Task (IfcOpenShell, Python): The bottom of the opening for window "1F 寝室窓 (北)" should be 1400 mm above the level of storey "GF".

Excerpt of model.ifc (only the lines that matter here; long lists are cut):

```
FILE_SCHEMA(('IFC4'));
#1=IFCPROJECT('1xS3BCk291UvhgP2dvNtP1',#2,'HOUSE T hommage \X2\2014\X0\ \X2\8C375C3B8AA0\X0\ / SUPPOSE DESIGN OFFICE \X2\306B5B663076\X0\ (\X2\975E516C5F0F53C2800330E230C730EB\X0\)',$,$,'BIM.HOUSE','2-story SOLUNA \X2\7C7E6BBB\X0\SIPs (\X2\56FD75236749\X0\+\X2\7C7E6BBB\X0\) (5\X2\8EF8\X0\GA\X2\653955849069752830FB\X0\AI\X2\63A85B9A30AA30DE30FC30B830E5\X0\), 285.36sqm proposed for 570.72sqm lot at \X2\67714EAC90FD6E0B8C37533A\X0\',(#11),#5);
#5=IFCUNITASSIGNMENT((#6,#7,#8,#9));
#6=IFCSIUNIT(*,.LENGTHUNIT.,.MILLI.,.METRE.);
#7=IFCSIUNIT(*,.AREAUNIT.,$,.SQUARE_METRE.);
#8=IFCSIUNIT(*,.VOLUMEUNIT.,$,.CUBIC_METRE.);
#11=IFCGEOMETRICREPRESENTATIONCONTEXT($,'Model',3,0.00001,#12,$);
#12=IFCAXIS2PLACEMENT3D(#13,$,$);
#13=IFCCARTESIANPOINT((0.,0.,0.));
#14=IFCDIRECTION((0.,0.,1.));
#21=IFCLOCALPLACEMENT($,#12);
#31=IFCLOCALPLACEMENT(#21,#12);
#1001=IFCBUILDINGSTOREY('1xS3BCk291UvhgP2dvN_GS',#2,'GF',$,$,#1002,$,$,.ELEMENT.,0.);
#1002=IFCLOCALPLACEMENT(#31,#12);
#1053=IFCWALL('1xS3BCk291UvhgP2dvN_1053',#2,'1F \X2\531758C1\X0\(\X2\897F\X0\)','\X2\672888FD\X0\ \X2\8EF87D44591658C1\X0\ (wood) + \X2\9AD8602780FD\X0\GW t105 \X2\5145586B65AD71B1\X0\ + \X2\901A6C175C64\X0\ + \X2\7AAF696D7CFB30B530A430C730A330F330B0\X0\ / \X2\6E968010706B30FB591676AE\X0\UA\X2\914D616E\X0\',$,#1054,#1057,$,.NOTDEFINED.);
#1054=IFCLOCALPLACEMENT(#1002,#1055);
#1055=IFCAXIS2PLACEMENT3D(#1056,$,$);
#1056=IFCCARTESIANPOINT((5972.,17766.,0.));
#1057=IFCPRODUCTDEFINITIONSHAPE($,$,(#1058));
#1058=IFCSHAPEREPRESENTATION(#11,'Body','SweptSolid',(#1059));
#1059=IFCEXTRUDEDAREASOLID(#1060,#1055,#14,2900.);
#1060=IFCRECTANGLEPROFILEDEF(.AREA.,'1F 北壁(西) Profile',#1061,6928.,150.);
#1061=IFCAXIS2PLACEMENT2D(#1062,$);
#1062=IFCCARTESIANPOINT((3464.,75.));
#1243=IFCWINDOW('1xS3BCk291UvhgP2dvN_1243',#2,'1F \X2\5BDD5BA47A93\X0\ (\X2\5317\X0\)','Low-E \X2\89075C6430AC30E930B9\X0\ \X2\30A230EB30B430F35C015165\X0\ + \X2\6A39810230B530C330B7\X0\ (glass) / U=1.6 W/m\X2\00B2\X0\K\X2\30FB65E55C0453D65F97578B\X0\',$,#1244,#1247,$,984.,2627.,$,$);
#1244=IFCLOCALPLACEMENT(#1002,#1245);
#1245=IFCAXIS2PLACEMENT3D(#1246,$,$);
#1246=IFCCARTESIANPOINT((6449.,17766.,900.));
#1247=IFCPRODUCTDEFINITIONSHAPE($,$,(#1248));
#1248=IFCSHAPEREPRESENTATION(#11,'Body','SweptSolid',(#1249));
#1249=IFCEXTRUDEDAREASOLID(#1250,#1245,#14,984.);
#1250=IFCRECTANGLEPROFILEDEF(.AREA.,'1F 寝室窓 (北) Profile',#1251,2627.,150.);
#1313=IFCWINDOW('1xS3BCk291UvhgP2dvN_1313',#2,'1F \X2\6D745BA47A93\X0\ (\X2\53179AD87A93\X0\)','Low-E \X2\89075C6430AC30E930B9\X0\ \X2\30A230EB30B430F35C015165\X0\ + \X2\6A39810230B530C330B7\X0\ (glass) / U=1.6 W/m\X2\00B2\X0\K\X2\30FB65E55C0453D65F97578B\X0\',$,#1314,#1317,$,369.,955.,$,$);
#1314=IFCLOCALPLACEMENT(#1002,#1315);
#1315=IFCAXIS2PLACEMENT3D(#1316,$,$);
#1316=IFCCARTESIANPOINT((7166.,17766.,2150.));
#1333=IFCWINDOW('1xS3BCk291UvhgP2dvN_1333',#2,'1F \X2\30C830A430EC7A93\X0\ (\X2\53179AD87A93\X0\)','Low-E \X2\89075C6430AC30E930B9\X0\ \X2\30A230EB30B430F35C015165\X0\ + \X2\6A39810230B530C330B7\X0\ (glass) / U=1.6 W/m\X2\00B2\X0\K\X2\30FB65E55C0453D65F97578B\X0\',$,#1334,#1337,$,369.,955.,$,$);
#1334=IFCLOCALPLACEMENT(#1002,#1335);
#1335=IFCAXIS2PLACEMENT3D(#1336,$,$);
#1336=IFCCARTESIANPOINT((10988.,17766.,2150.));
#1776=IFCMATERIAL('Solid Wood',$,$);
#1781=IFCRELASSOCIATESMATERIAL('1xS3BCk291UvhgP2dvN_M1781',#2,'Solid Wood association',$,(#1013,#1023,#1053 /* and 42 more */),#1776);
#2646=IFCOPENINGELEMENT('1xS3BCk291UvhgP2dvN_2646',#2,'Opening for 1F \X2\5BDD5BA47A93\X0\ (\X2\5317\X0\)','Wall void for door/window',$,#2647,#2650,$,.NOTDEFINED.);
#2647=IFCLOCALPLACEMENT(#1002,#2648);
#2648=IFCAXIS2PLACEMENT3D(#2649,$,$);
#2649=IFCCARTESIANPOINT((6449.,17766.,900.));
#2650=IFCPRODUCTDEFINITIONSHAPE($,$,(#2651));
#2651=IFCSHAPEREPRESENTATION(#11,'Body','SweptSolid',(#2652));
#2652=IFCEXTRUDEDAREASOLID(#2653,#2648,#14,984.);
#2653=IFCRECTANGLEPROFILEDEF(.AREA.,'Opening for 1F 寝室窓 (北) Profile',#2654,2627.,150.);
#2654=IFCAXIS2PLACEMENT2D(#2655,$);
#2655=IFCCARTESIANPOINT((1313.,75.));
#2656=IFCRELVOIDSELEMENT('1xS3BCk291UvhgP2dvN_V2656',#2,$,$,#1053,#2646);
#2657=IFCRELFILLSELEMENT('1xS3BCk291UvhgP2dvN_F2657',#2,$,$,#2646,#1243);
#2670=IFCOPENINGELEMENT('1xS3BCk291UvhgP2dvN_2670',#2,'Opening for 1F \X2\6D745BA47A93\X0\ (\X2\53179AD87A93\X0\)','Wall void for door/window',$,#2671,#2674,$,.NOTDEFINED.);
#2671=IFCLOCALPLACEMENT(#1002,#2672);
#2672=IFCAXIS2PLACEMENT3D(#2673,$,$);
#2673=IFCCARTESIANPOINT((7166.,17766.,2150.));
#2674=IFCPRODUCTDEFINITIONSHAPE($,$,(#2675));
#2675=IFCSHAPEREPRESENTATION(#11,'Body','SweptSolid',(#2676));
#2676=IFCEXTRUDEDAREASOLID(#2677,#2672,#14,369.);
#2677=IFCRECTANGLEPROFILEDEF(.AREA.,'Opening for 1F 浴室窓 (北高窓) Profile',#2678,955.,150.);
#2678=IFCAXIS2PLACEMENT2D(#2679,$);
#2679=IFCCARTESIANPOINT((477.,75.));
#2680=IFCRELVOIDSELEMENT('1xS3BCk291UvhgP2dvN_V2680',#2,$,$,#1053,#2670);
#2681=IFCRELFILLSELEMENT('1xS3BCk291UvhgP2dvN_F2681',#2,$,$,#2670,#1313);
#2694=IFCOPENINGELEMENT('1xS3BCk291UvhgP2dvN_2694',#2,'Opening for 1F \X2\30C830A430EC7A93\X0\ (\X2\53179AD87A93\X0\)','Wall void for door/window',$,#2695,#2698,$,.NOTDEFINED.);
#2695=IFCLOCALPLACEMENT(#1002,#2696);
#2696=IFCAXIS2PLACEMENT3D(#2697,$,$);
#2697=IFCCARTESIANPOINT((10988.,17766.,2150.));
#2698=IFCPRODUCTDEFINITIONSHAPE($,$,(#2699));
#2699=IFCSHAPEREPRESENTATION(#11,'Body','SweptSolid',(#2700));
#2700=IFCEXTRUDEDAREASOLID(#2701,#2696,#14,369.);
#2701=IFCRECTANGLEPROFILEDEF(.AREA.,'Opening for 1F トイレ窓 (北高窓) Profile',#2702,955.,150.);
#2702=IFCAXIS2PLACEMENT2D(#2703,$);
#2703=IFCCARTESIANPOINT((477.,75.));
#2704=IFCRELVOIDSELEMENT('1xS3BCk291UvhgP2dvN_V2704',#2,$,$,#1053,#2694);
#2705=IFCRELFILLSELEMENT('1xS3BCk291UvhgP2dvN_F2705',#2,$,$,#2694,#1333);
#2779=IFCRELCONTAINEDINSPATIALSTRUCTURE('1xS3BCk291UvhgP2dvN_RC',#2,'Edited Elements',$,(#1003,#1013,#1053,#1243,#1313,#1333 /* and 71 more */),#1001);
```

```python
import numpy as np
import ifcopenshell
import ifcopenshell.api.geometry
import ifcopenshell.geom
import ifcopenshell.util.element
import ifcopenshell.util.placement
import ifcopenshell.util.shape
import ifcopenshell.util.unit

model = ifcopenshell.open("model.ifc")
unit_scale = ifcopenshell.util.unit.calculate_unit_scale(model)

window = model.by_id(1243)
opening = window.FillsVoids[0].RelatingOpeningElement
storey = ifcopenshell.util.element.get_container(window, ifc_class="IfcBuildingStorey")
level = ifcopenshell.util.placement.get_local_placement(storey.ObjectPlacement)[2, 3]

# The opening's origin need not be at the sill, so measure its lowest point.
shape = ifcopenshell.geom.create_shape(ifcopenshell.geom.settings(), opening)
bottom = ifcopenshell.util.shape.get_shape_bottom_elevation(shape, shape.geometry) / unit_scale
dz = level + 1400.0 - bottom

shift = np.array([0.0, 0.0, dz])
# The window is not placed relative to its opening, so move both.
for product in (opening, window):
    matrix = ifcopenshell.util.placement.get_local_placement(product.ObjectPlacement)
    matrix[:3, 3] += shift
    ifcopenshell.api.geometry.edit_object_placement(model, product=product, matrix=matrix, is_si=False)

print(f"moved by {dz * unit_scale:+.3f} m")

model.write("model_updated.ifc")
```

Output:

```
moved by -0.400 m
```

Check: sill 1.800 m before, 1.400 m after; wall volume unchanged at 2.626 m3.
